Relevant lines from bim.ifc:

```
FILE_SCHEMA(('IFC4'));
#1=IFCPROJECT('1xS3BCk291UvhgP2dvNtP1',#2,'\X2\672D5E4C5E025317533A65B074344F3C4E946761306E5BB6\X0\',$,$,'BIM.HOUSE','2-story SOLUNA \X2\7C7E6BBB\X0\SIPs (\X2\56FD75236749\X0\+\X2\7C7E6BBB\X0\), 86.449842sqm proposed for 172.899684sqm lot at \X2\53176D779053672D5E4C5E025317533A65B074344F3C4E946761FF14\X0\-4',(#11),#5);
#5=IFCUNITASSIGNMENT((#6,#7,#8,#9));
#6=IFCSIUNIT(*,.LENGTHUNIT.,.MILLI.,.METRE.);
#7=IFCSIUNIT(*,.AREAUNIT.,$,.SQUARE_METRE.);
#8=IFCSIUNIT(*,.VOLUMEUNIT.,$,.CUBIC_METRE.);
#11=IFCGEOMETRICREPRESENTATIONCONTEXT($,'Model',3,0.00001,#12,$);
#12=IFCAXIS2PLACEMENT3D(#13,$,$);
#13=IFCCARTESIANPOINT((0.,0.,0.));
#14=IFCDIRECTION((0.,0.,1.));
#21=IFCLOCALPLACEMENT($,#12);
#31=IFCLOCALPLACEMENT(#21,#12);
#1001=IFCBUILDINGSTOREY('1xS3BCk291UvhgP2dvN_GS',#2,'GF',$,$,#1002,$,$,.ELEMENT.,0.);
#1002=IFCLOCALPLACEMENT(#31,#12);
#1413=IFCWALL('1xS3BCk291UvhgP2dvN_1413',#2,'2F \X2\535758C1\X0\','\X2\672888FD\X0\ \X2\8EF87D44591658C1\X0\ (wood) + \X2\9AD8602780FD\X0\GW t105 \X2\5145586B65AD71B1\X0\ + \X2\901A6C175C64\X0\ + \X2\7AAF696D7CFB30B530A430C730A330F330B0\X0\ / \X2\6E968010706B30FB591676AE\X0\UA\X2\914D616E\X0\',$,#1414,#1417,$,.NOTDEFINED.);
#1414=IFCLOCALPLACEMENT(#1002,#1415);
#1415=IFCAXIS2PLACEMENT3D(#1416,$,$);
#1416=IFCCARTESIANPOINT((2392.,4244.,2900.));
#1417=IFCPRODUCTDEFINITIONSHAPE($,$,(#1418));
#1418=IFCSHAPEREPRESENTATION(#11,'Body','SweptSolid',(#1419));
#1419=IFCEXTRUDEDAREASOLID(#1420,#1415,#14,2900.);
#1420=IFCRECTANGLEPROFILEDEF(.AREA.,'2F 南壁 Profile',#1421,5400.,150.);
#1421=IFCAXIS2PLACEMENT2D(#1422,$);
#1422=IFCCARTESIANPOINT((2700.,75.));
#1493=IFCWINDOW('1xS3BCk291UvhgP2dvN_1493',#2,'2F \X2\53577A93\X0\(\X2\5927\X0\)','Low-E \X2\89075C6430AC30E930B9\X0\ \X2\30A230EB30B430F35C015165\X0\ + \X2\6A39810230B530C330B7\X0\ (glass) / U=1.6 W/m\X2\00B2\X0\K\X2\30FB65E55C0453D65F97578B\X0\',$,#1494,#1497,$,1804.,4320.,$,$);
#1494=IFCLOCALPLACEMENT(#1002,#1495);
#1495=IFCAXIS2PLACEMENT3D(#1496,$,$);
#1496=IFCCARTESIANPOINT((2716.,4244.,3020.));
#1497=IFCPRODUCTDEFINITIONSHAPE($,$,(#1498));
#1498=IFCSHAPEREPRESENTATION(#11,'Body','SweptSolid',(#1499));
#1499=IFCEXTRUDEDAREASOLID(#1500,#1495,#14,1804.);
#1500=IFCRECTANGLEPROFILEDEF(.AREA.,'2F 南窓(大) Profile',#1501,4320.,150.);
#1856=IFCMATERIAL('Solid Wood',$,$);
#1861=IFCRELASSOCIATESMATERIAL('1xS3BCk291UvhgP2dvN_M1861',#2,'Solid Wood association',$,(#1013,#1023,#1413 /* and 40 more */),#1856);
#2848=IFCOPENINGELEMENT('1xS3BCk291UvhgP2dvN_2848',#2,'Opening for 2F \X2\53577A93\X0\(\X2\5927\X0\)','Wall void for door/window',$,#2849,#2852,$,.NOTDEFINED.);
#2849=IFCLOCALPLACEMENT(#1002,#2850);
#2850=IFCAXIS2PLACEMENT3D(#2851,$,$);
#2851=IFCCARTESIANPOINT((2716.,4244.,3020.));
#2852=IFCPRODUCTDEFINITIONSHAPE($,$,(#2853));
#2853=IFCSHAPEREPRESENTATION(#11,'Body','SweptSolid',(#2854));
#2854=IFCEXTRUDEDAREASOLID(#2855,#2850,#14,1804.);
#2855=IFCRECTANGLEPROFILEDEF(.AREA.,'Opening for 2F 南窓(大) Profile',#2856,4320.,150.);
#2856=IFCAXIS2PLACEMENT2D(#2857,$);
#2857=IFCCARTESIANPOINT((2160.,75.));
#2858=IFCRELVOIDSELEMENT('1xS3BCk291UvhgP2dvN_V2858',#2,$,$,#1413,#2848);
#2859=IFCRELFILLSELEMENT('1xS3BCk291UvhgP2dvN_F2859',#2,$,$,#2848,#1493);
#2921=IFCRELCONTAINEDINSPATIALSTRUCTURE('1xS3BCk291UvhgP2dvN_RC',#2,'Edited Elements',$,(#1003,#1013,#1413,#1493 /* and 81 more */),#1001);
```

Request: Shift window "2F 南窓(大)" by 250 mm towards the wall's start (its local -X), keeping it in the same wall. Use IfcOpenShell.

```python
import ifcopenshell
import ifcopenshell.api.geometry
import ifcopenshell.util.placement
import ifcopenshell.util.unit

model = ifcopenshell.open("bim.ifc")
unit_scale = ifcopenshell.util.unit.calculate_unit_scale(model)

window = model.by_guid("1xS3BCk291UvhgP2dvN_1493")
opening = window.FillsVoids[0].RelatingOpeningElement
wall = opening.VoidsElements[0].RelatingBuildingElement

wall_matrix = ifcopenshell.util.placement.get_local_placement(wall.ObjectPlacement)
shift = wall_matrix[:3, 0] * -0.25 / unit_scale
before = ifcopenshell.util.placement.get_local_placement(window.ObjectPlacement)[:3, 3].copy()

# The window is not placed relative to its opening, so move both.
for product in (opening, window):
    matrix = ifcopenshell.util.placement.get_local_placement(product.ObjectPlacement)
    matrix[:3, 3] += shift
    ifcopenshell.api.geometry.edit_object_placement(model, product=product, matrix=matrix, is_si=False)

after = ifcopenshell.util.placement.get_local_placement(window.ObjectPlacement)[:3, 3]
print("window moved by", (after - before).round(3) + 0.0)

model.write("bim_updated.ifc")
```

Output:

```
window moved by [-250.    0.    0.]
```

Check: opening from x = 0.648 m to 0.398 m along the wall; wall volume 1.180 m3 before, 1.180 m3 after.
